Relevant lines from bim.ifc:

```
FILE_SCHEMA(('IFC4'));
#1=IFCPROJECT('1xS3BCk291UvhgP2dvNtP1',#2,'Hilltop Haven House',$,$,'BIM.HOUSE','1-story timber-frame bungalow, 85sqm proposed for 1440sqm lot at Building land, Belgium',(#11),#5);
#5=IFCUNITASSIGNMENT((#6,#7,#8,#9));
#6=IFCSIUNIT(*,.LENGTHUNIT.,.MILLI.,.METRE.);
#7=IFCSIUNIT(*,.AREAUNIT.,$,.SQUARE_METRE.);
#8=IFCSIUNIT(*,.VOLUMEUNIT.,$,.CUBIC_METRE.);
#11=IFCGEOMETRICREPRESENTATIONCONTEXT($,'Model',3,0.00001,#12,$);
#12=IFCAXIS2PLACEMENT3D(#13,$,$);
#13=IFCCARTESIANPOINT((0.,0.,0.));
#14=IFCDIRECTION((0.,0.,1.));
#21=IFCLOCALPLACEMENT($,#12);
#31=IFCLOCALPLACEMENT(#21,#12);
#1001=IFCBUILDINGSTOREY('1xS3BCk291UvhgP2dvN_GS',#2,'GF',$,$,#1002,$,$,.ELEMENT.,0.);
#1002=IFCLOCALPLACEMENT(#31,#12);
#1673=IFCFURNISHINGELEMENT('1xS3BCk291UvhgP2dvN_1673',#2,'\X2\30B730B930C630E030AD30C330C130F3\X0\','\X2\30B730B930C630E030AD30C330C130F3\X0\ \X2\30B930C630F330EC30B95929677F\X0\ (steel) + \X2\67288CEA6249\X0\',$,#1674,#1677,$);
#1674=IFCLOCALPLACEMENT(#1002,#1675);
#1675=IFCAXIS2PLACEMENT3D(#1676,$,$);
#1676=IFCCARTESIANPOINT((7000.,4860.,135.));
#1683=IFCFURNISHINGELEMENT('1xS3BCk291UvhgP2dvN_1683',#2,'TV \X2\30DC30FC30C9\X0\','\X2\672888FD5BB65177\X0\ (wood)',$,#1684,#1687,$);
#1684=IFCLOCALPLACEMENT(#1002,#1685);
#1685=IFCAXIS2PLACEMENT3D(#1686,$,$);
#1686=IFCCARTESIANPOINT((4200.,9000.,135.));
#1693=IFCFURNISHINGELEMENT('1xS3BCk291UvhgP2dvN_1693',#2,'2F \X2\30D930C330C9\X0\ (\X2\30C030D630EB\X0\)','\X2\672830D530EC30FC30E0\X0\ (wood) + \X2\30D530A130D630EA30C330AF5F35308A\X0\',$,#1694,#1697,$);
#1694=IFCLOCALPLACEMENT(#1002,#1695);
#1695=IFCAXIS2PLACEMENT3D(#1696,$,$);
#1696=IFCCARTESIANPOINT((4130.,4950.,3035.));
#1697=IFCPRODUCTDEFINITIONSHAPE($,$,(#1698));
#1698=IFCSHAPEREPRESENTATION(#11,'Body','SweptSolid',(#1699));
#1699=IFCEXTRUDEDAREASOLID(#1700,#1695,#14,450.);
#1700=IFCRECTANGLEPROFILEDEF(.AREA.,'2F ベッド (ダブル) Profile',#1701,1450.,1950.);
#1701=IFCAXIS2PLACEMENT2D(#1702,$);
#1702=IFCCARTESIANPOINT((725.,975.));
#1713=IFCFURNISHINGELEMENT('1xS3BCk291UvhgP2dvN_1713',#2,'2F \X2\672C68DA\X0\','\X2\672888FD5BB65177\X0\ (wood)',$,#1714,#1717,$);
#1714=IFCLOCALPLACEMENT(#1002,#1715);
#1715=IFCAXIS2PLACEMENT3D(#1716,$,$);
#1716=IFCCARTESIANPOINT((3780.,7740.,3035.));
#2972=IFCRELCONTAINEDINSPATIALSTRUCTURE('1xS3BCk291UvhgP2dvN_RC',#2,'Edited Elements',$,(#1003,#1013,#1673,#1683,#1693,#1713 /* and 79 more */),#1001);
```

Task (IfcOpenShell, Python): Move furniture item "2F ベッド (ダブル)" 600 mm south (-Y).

```python
import ifcopenshell
import ifcopenshell.api.geometry
import ifcopenshell.util.placement
import ifcopenshell.util.unit

model = ifcopenshell.open("bim.ifc")
unit_scale = ifcopenshell.util.unit.calculate_unit_scale(model)

item = model.by_guid("1xS3BCk291UvhgP2dvN_1693")
matrix = ifcopenshell.util.placement.get_local_placement(item.ObjectPlacement)
matrix[1, 3] -= 0.6 / unit_scale
ifcopenshell.api.geometry.edit_object_placement(model, product=item, matrix=matrix, is_si=False)

print(ifcopenshell.util.placement.get_local_placement(item.ObjectPlacement).round(3) + 0.0)

model.write("bim_v2.ifc")
```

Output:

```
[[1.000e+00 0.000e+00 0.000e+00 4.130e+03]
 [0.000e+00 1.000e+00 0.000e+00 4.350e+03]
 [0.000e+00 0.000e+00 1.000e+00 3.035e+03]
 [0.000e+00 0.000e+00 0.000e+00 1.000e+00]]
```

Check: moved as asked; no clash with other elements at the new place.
